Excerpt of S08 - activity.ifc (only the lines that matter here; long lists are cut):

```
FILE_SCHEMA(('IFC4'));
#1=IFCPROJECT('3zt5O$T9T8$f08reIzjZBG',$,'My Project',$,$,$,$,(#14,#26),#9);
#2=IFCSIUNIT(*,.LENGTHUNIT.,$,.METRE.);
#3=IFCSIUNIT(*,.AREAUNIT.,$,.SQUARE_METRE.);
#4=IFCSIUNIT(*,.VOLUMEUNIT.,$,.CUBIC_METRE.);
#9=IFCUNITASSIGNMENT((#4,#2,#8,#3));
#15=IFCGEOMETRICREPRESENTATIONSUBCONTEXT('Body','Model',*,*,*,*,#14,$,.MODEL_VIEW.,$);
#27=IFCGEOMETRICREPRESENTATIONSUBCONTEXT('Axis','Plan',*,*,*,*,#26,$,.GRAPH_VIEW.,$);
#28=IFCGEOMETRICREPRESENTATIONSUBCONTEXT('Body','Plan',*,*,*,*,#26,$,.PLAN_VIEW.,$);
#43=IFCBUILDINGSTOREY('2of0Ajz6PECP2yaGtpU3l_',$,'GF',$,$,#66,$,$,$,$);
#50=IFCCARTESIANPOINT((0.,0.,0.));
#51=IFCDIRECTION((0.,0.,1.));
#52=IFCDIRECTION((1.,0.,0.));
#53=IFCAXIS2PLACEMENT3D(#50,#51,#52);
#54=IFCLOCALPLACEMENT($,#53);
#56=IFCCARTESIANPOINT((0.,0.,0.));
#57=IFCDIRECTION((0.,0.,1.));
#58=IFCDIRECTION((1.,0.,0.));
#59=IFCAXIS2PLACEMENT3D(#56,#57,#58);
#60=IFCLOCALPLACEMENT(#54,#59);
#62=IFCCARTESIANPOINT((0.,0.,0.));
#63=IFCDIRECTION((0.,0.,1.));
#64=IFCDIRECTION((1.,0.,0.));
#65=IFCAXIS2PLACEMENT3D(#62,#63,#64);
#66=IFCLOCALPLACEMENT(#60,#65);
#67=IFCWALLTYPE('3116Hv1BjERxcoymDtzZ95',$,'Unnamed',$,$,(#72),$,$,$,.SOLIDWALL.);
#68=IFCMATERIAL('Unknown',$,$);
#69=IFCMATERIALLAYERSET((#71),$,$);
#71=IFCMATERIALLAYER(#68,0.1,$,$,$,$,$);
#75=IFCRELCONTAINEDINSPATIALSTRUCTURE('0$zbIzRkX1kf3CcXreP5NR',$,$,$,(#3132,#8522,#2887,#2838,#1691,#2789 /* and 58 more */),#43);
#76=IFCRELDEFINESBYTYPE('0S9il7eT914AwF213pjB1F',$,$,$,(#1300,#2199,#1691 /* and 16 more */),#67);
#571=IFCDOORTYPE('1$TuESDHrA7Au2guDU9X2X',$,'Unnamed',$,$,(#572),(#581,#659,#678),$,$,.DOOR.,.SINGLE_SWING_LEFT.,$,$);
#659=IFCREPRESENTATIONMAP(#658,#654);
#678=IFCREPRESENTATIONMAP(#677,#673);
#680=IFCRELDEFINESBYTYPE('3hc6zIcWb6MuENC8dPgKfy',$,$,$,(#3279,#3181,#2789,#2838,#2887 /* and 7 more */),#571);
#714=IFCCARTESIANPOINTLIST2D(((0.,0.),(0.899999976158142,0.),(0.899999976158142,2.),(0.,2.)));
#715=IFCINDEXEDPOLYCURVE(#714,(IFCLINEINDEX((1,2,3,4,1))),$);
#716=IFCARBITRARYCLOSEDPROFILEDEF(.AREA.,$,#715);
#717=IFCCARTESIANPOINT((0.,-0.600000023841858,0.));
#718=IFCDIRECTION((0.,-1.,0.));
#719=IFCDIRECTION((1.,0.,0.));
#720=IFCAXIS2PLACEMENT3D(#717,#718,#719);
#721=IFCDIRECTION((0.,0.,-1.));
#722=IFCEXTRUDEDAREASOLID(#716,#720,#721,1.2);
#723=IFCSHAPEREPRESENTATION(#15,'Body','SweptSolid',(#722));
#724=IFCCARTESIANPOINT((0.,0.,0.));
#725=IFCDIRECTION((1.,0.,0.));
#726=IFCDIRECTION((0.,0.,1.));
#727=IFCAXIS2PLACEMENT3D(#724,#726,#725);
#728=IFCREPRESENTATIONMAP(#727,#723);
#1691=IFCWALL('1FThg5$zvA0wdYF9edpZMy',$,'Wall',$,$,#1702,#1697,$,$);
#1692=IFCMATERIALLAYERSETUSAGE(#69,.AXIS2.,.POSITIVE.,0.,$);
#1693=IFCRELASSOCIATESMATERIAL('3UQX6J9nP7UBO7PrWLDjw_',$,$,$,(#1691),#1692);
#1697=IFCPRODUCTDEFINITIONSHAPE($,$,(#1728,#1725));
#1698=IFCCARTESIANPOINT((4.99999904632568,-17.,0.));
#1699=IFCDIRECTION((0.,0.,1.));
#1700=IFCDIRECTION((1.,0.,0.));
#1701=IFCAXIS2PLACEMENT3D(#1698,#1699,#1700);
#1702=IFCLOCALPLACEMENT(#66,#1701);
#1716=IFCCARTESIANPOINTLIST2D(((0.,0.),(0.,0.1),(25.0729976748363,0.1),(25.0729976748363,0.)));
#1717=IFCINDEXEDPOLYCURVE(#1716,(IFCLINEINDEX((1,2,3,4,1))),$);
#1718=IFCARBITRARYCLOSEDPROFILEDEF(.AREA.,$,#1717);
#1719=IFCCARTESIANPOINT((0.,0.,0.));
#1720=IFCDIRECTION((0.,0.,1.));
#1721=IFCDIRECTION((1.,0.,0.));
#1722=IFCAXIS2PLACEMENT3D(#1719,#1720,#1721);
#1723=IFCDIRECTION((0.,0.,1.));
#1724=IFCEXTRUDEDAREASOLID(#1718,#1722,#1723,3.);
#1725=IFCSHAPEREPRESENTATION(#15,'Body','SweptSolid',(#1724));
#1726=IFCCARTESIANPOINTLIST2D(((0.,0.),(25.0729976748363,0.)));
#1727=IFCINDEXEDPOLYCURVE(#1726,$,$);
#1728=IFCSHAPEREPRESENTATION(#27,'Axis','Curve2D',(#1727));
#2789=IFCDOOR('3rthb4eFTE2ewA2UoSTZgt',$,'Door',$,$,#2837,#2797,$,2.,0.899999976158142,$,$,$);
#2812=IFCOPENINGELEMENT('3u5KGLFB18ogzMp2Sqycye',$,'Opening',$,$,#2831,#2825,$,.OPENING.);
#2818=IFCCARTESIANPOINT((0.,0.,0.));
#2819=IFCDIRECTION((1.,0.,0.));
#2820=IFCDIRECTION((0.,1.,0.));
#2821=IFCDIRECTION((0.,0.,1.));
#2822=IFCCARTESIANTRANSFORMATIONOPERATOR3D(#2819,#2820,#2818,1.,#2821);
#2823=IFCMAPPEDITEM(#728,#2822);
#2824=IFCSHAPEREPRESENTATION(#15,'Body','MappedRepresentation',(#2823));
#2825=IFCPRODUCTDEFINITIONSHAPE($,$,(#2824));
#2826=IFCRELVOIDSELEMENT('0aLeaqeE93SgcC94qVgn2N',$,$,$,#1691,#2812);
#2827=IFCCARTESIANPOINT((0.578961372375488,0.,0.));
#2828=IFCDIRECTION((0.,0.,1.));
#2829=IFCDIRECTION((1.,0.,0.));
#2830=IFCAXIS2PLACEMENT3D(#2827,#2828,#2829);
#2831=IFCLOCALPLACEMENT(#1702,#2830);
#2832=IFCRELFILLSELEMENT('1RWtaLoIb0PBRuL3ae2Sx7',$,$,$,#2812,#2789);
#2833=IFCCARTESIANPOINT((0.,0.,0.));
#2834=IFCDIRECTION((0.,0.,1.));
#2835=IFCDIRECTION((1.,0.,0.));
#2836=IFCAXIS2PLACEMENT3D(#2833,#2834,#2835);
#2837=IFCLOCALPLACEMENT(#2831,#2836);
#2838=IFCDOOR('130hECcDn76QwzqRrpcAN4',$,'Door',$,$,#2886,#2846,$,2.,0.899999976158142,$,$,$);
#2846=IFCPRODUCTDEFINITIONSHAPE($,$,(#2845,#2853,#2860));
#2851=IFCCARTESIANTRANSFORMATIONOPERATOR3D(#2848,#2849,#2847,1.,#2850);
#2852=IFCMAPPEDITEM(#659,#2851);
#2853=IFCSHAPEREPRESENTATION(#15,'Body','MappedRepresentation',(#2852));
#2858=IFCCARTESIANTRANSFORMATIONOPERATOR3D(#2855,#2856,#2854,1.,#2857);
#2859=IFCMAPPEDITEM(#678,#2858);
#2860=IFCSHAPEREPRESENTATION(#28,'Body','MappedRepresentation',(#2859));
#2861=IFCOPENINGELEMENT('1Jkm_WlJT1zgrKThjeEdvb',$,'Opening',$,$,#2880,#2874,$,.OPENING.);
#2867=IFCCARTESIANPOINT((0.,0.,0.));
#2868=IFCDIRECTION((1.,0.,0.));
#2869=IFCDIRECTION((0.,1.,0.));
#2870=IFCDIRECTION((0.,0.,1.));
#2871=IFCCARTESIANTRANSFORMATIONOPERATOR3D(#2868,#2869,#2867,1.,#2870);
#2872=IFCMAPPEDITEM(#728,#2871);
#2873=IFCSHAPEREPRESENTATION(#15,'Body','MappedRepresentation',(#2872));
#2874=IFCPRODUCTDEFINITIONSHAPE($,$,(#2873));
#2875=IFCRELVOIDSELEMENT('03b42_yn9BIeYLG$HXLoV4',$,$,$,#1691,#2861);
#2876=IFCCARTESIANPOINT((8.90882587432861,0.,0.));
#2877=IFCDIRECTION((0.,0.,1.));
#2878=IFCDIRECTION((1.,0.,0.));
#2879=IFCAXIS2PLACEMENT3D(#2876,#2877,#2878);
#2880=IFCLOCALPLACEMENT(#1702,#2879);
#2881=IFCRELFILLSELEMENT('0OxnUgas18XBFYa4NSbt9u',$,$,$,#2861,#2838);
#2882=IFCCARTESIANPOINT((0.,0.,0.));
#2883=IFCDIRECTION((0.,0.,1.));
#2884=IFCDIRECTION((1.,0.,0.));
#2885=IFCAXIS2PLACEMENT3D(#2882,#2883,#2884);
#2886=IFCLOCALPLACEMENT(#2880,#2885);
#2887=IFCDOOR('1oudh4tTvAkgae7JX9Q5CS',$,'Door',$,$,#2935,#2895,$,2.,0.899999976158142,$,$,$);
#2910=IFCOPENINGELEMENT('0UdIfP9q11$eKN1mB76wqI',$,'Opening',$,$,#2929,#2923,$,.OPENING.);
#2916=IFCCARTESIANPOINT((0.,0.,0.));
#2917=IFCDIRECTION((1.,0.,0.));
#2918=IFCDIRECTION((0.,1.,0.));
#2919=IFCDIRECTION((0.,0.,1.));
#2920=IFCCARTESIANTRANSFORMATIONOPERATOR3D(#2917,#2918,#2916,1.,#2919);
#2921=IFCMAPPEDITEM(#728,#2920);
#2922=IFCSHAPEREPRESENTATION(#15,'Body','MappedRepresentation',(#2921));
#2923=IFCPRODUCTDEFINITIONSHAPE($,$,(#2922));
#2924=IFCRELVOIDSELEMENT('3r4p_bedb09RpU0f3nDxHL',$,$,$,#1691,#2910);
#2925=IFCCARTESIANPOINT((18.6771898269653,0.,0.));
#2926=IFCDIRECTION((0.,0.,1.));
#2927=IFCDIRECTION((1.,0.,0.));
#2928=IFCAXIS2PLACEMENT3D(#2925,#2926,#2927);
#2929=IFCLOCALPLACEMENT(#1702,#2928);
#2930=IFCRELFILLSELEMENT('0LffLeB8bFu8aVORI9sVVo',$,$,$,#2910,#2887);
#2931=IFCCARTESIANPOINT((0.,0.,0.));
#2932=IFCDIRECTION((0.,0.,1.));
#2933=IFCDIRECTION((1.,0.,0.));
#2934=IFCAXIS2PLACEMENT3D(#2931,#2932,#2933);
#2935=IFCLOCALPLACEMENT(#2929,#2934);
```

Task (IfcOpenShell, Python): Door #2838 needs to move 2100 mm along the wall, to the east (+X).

```python
import ifcopenshell
import ifcopenshell.api.geometry
import ifcopenshell.util.placement
import ifcopenshell.util.unit

model = ifcopenshell.open("S08 - activity.ifc")
unit_scale = ifcopenshell.util.unit.calculate_unit_scale(model)

door = model.by_id(2838)
opening = door.FillsVoids[0].RelatingOpeningElement
wall = opening.VoidsElements[0].RelatingBuildingElement

wall_matrix = ifcopenshell.util.placement.get_local_placement(wall.ObjectPlacement)
shift = wall_matrix[:3, 0] * 2.1 / unit_scale
before = ifcopenshell.util.placement.get_local_placement(door.ObjectPlacement)[:3, 3].copy()

# The door is placed relative to its opening, so it follows when the opening moves.
matrix = ifcopenshell.util.placement.get_local_placement(opening.ObjectPlacement)
matrix[:3, 3] += shift
ifcopenshell.api.geometry.edit_object_placement(
    model, product=opening, matrix=matrix, is_si=False, should_transform_children=True
)

after = ifcopenshell.util.placement.get_local_placement(door.ObjectPlacement)[:3, 3]
print("door moved by", (after - before).round(3) + 0.0)

model.write("S08 - activity_updated.ifc")
```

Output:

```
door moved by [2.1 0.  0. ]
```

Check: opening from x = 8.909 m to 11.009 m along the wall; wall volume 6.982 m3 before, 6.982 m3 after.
